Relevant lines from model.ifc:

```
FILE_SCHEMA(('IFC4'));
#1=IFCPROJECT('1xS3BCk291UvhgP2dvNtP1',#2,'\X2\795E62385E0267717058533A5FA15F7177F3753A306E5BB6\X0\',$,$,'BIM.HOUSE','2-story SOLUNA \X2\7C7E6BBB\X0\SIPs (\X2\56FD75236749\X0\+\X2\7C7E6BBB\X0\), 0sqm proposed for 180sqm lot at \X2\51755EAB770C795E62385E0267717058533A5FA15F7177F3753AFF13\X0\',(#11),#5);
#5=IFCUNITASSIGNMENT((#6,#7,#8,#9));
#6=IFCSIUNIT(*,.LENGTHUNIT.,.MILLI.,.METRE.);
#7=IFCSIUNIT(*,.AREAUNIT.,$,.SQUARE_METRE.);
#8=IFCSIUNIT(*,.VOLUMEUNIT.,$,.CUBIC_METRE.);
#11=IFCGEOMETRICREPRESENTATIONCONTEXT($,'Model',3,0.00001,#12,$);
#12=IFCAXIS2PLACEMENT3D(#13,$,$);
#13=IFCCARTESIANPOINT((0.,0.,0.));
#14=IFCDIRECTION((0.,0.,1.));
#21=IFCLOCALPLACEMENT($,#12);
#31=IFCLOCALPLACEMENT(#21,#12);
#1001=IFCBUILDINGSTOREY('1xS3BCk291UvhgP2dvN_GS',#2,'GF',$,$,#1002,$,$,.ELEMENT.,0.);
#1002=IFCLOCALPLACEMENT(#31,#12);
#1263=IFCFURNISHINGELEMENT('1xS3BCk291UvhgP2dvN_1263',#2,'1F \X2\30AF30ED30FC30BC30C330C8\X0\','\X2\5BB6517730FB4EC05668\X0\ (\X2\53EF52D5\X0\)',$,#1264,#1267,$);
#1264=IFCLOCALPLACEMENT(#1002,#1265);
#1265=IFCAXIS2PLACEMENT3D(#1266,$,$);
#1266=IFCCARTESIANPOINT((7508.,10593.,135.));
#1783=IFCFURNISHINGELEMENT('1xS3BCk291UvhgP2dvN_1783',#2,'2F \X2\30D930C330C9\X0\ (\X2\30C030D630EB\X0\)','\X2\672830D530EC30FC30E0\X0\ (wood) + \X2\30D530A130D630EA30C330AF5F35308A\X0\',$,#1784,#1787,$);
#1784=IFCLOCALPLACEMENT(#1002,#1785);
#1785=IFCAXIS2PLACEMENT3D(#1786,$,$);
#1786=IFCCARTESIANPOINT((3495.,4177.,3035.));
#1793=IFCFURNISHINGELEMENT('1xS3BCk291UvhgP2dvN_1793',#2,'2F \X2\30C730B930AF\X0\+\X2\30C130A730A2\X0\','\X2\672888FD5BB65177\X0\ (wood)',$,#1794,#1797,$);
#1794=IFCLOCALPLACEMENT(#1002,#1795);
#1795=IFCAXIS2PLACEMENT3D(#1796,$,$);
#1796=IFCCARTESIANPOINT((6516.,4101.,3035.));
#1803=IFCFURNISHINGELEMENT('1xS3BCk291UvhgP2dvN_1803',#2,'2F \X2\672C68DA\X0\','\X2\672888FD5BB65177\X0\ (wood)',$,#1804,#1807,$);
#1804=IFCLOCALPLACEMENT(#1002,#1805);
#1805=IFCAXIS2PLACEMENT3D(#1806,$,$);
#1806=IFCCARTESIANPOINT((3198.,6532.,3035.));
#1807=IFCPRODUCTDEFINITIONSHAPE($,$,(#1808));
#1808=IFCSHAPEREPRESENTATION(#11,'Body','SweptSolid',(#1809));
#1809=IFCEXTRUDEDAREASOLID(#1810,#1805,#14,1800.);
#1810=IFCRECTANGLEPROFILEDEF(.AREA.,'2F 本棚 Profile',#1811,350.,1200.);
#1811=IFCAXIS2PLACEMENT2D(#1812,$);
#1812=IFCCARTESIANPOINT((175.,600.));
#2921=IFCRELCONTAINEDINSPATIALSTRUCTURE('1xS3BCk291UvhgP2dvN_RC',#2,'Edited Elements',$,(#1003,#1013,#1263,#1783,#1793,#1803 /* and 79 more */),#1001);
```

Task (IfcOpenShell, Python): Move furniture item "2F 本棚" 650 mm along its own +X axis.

```python
import ifcopenshell
import ifcopenshell.api.geometry
import ifcopenshell.util.placement
import ifcopenshell.util.unit

model = ifcopenshell.open("model.ifc")
unit_scale = ifcopenshell.util.unit.calculate_unit_scale(model)

item = model.by_id(1803)
matrix = ifcopenshell.util.placement.get_local_placement(item.ObjectPlacement)
matrix[:3, 3] += matrix[:3, 0] * 0.65 / unit_scale
ifcopenshell.api.geometry.edit_object_placement(model, product=item, matrix=matrix, is_si=False)

print(ifcopenshell.util.placement.get_local_placement(item.ObjectPlacement).round(3) + 0.0)

model.write("model_rev.ifc")
```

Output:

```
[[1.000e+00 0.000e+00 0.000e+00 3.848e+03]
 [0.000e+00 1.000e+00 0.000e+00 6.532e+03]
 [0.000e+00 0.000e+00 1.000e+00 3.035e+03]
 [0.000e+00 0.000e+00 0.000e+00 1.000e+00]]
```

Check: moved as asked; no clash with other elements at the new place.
